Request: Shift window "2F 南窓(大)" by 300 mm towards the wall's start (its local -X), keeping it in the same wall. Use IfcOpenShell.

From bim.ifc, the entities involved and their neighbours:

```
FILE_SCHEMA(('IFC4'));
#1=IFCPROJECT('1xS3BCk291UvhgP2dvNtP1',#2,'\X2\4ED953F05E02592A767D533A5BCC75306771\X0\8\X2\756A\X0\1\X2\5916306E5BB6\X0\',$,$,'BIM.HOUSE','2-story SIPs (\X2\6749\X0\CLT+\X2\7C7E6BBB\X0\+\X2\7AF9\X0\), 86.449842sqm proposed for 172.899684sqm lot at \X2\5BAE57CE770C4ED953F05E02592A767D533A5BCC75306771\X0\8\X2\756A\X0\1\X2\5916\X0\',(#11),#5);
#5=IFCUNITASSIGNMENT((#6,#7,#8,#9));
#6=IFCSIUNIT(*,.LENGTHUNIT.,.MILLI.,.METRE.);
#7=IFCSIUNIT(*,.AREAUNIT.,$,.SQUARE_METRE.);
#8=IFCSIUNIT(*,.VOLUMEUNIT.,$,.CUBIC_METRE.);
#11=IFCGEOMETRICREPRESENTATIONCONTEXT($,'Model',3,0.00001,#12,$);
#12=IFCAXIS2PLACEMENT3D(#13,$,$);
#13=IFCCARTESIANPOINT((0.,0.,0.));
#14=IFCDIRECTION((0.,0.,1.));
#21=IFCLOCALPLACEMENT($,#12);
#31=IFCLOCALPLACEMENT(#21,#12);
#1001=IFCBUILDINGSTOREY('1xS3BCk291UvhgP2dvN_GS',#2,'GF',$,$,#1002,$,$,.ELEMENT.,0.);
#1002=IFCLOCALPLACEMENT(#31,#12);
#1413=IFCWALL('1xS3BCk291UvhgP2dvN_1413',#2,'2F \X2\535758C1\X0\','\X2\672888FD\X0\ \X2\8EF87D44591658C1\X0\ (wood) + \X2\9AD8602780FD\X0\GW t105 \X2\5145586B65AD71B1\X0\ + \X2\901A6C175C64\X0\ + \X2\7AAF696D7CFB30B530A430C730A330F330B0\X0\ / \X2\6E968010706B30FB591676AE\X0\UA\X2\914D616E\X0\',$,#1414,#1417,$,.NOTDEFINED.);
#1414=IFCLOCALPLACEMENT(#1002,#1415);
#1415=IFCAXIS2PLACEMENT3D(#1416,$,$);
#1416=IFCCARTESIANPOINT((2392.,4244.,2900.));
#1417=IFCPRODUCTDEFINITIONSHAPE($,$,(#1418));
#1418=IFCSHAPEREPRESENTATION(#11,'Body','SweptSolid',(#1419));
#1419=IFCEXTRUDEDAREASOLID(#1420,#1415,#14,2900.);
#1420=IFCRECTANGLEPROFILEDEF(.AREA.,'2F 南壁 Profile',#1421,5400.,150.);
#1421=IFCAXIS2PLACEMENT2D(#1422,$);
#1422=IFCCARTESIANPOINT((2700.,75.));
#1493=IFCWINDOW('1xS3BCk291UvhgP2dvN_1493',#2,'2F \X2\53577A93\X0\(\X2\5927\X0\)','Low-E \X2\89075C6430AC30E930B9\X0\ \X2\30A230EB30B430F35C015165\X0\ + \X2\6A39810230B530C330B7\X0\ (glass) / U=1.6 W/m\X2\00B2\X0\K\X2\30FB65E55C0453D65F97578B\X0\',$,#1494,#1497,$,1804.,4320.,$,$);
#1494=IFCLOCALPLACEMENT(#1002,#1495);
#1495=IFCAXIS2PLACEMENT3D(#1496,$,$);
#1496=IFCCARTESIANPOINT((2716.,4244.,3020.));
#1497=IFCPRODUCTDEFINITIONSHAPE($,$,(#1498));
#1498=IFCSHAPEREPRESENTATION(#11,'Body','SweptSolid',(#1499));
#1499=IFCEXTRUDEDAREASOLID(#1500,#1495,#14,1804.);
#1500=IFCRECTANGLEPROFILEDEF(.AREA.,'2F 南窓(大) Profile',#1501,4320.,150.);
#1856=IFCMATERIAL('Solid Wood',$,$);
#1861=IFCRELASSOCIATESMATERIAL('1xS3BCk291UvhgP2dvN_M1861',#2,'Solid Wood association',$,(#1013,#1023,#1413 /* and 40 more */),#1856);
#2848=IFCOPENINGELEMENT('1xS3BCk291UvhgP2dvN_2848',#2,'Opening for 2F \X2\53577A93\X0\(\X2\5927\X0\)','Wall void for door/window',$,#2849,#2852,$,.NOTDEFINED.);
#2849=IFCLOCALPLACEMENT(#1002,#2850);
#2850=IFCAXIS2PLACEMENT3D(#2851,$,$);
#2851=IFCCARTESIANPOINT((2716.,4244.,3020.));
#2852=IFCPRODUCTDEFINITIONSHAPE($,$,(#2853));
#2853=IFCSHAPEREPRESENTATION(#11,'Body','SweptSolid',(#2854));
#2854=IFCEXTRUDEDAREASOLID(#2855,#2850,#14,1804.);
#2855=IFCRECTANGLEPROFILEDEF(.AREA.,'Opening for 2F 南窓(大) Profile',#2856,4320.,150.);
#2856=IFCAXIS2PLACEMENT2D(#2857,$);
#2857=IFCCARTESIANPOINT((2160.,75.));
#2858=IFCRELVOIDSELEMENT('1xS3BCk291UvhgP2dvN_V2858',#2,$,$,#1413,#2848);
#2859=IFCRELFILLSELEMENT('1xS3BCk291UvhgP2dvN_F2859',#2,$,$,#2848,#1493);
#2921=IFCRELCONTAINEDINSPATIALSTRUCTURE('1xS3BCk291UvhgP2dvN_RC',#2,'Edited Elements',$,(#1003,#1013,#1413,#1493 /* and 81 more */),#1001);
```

```python
import ifcopenshell
import ifcopenshell.api.geometry
import ifcopenshell.util.placement

model = ifcopenshell.open("bim.ifc")

window = model.by_id(1493)
opening = window.FillsVoids[0].RelatingOpeningElement
wall = opening.VoidsElements[0].RelatingBuildingElement

wall_matrix = ifcopenshell.util.placement.get_local_placement(wall.ObjectPlacement)
shift = wall_matrix[:3, 0] * -300.0
before = ifcopenshell.util.placement.get_local_placement(window.ObjectPlacement)[:3, 3].copy()

# The window is not placed relative to its opening, so move both.
for product in (opening, window):
    matrix = ifcopenshell.util.placement.get_local_placement(product.ObjectPlacement)
    matrix[:3, 3] += shift
    ifcopenshell.api.geometry.edit_object_placement(model, product=product, matrix=matrix, is_si=False)

after = ifcopenshell.util.placement.get_local_placement(window.ObjectPlacement)[:3, 3]
print("window moved by", (after - before).round(3) + 0.0)

model.write("bim_v2.ifc")
```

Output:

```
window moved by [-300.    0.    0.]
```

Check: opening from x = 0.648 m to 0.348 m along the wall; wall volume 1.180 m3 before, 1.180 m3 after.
